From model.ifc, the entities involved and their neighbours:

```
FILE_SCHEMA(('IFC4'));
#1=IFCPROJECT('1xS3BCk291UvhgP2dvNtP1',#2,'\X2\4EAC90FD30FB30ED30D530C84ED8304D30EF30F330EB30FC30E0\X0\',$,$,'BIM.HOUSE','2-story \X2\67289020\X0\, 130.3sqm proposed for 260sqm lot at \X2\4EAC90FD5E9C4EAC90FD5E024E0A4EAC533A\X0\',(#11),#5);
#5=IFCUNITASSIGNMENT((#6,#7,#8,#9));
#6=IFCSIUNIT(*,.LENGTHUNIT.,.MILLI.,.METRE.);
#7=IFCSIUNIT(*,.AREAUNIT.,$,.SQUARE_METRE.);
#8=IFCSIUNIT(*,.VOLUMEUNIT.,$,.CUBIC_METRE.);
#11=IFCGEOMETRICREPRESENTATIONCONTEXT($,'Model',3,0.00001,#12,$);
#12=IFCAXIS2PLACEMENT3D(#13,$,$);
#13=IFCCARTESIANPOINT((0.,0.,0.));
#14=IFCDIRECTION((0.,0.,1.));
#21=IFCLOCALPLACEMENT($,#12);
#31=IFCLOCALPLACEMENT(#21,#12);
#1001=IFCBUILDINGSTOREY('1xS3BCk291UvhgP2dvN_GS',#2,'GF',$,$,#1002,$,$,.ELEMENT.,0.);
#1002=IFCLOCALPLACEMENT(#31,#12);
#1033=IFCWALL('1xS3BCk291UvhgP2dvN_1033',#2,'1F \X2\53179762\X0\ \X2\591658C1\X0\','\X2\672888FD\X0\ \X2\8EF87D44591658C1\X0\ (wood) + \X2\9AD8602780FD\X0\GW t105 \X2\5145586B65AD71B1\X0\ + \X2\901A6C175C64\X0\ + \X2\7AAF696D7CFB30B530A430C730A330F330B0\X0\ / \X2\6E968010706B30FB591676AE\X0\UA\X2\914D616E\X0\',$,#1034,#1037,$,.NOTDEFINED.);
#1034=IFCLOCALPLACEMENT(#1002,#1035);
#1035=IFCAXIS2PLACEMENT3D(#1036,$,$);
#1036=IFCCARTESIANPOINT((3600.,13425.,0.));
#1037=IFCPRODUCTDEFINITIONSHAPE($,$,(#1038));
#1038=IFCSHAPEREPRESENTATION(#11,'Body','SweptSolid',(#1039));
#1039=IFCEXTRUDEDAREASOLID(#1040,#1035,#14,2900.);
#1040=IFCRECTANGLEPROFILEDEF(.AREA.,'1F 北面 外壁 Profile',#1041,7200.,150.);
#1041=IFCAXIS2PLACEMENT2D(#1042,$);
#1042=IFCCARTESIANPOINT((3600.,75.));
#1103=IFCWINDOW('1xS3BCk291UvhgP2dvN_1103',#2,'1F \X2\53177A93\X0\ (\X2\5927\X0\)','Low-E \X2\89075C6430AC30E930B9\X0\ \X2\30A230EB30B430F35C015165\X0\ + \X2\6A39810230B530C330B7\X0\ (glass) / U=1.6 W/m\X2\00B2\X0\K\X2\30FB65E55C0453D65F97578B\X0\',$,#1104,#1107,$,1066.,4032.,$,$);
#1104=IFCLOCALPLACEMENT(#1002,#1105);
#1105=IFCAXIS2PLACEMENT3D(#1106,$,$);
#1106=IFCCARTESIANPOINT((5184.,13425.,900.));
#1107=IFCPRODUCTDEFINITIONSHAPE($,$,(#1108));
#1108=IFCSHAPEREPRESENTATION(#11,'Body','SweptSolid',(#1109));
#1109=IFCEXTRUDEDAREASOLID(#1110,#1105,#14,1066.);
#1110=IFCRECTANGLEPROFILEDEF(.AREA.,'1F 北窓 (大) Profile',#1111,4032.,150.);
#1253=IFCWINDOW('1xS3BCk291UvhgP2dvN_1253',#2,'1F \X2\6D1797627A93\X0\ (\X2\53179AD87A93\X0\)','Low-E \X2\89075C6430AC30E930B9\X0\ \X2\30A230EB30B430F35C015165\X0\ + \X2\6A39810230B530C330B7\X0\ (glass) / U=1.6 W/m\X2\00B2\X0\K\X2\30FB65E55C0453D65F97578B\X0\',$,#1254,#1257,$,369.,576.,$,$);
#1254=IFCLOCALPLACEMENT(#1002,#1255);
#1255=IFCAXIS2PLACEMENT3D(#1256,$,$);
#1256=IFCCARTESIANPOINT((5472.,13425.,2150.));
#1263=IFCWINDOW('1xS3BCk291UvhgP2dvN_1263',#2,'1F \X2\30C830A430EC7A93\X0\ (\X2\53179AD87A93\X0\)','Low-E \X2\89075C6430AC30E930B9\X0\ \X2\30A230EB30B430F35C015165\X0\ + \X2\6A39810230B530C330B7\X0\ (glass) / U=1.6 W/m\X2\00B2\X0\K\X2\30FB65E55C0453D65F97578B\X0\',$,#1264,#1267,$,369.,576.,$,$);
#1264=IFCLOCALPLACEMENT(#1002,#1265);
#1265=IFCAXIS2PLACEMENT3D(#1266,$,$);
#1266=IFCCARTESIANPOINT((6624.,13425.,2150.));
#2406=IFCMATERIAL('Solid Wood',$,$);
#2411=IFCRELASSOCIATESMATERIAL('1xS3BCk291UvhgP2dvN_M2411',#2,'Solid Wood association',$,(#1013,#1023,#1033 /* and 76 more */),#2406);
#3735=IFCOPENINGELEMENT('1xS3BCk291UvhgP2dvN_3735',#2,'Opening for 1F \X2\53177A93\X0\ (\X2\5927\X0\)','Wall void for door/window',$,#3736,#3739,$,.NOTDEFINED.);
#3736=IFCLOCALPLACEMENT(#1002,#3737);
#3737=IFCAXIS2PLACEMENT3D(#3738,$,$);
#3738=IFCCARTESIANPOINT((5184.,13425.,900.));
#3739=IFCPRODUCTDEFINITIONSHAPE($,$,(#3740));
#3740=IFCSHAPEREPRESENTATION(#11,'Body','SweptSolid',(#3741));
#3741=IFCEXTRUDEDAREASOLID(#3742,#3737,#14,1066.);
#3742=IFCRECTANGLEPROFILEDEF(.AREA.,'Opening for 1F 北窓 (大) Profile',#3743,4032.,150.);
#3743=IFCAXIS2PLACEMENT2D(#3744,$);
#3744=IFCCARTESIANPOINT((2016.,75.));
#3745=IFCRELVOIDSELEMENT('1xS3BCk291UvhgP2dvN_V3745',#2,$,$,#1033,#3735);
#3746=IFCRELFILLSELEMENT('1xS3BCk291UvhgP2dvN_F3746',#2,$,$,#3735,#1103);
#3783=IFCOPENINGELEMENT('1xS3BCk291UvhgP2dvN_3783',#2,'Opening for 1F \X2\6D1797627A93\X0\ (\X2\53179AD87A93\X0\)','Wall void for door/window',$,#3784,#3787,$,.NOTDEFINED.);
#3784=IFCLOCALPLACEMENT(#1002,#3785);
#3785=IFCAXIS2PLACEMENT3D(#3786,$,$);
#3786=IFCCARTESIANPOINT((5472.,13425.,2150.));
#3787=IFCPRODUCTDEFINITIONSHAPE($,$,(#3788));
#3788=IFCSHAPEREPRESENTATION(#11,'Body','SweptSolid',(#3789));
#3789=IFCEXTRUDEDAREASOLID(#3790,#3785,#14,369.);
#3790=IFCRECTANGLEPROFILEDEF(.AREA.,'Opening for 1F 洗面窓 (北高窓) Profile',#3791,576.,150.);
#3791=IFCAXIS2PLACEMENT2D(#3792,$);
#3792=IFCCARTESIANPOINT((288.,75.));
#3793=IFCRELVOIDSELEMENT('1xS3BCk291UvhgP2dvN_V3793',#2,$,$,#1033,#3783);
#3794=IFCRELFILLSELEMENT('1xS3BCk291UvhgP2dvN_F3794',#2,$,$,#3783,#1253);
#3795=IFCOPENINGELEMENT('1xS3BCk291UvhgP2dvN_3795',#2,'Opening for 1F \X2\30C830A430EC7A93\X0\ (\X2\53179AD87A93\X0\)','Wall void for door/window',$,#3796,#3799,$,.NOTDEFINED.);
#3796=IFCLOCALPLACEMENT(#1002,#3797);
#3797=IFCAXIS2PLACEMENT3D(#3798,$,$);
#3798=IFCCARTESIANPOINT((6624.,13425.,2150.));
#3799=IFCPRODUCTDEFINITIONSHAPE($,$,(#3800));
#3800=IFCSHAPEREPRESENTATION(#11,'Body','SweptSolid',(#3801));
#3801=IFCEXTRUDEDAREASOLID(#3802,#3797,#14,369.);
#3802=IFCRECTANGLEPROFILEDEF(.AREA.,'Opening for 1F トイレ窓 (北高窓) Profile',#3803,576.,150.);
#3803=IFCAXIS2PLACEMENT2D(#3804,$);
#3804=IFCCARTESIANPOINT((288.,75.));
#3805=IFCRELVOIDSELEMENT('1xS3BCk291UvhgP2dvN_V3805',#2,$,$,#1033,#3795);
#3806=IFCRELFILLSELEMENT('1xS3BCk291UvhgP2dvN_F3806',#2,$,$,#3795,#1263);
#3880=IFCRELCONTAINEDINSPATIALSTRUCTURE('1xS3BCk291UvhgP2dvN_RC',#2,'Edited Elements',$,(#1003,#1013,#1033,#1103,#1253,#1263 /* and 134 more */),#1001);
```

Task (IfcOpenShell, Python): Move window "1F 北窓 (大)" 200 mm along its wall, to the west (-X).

```python
import ifcopenshell
import ifcopenshell.api.geometry
import ifcopenshell.util.placement
import ifcopenshell.util.unit

model = ifcopenshell.open("model.ifc")
unit_scale = ifcopenshell.util.unit.calculate_unit_scale(model)

window = model.by_guid("1xS3BCk291UvhgP2dvN_1103")
opening = window.FillsVoids[0].RelatingOpeningElement
wall = opening.VoidsElements[0].RelatingBuildingElement

wall_matrix = ifcopenshell.util.placement.get_local_placement(wall.ObjectPlacement)
shift = wall_matrix[:3, 0] * -0.2 / unit_scale
before = ifcopenshell.util.placement.get_local_placement(window.ObjectPlacement)[:3, 3].copy()

# The window is not placed relative to its opening, so move both.
for product in (opening, window):
    matrix = ifcopenshell.util.placement.get_local_placement(product.ObjectPlacement)
    matrix[:3, 3] += shift
    ifcopenshell.api.geometry.edit_object_placement(model, product=product, matrix=matrix, is_si=False)

after = ifcopenshell.util.placement.get_local_placement(window.ObjectPlacement)[:3, 3]
print("window moved by", (after - before).round(3) + 0.0)

model.write("model_edited.ifc")
```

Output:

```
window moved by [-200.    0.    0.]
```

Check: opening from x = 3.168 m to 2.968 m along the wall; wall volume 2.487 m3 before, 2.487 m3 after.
